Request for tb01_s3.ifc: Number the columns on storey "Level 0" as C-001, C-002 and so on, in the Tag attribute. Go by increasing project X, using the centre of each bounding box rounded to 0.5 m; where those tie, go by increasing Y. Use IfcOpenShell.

First a look at what the model holds.

```python
import ifcopenshell
import ifcopenshell.util.element
import ifcopenshell.util.placement

model = ifcopenshell.open("tb01_s3.ifc")
print(model.schema)
storey = next(s for s in model.by_type("IfcBuildingStorey") if s.Name == "Level 0")
columns = [e for e in ifcopenshell.util.element.get_decomposition(storey) if e.is_a("IfcColumn")]
for e in sorted(columns, key=lambda e: e.id()):
    origin = ifcopenshell.util.placement.get_local_placement(e.ObjectPlacement)[:3, 3]
    print(e.id(), e.Tag, e.Name, origin.round(2) + 0.0, sep=" | ")
```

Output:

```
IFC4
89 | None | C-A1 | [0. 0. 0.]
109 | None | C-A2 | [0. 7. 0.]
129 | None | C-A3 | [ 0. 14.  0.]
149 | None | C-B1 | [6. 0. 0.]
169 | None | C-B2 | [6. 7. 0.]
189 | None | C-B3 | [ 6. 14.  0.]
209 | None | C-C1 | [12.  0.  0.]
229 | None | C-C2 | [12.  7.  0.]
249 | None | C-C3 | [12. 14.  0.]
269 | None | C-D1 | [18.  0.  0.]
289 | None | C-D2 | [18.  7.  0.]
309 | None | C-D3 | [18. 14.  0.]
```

```python
import ifcopenshell
import ifcopenshell.geom
import ifcopenshell.util.element
import ifcopenshell.util.shape

model = ifcopenshell.open("tb01_s3.ifc")
settings = ifcopenshell.geom.settings()
settings.set("use-world-coords", True)


def centre(element):
    shape = ifcopenshell.geom.create_shape(settings, element)
    return ifcopenshell.util.shape.get_bbox_centroid(shape.geometry)


storey = next(s for s in model.by_type("IfcBuildingStorey") if s.Name == "Level 0")
columns = [e for e in ifcopenshell.util.element.get_decomposition(storey) if e.is_a("IfcColumn")]

# Insertion points can sit at a corner or the storey origin, so sort by the geometry (in metres).
centres = {e: centre(e) for e in columns}
columns.sort(key=lambda e: (round(centres[e][0] / 0.5), centres[e][1]))

for i, e in enumerate(columns, start=1):
    number = f"C-0{i:02d}"
    e.Tag = number
    print(e.id(), number)

model.write("tb01_s3_v2.ifc")
```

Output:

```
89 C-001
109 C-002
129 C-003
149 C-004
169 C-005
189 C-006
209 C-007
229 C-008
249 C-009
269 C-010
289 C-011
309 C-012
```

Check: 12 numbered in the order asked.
